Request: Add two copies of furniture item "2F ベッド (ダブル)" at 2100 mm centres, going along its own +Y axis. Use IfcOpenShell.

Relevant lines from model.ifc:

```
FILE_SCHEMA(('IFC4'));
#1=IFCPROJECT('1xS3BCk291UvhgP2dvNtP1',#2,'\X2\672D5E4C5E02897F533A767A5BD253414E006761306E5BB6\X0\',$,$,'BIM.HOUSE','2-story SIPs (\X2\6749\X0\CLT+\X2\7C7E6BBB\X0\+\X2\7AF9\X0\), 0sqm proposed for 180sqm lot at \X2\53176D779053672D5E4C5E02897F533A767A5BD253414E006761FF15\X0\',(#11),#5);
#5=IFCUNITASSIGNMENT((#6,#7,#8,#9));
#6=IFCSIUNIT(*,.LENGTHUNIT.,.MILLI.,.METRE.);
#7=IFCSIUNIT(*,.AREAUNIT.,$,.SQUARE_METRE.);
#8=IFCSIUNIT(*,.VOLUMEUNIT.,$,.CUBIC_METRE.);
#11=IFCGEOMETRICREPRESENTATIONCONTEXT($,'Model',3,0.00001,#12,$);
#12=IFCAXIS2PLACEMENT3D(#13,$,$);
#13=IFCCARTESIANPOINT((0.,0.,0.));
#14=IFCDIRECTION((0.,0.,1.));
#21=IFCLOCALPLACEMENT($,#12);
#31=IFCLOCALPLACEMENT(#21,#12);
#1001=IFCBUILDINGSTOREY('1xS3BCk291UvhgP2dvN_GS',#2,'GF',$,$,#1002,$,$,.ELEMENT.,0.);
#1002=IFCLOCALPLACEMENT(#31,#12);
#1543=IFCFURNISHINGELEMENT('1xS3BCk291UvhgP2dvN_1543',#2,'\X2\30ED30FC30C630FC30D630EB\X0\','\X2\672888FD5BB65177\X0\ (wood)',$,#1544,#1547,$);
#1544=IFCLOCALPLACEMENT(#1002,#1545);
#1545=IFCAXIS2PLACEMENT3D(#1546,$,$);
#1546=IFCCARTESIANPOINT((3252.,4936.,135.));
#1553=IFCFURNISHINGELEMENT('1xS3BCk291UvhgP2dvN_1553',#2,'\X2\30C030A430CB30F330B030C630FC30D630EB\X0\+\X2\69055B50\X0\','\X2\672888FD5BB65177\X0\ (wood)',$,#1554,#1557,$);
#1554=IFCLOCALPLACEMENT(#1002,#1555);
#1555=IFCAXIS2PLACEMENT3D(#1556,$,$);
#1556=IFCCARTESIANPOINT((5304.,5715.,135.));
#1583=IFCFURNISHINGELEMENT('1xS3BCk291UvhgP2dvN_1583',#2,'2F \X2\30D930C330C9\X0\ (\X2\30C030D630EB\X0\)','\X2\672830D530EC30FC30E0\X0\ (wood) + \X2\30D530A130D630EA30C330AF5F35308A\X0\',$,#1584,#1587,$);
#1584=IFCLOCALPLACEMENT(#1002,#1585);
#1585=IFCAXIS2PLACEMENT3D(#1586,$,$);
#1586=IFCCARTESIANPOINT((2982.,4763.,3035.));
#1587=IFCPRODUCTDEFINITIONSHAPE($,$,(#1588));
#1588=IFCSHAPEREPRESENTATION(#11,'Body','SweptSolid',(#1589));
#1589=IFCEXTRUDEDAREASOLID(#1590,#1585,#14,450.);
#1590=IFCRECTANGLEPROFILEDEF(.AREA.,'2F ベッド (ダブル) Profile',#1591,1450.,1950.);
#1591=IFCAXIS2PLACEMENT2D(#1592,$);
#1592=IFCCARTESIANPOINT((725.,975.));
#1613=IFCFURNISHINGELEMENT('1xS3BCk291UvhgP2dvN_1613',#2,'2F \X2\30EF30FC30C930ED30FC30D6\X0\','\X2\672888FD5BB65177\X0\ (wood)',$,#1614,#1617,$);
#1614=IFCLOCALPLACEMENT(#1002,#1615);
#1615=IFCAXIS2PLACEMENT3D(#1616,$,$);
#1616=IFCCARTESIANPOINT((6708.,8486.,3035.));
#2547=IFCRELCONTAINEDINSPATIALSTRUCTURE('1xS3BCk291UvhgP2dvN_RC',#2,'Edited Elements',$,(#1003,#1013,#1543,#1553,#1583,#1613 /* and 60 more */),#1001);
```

```python
import ifcopenshell
import ifcopenshell.api.geometry
import ifcopenshell.api.root
import ifcopenshell.util.element
import ifcopenshell.util.placement

model = ifcopenshell.open("model.ifc")


def reuse_history(source, copy):
    """copy_class also copies each property set's owner history, people and application; keep the originals."""
    for rel in copy.IsDefinedBy:
        if rel.is_a("IfcRelDefinesByProperties") and (history := rel.RelatingPropertyDefinition.OwnerHistory):
            rel.RelatingPropertyDefinition.OwnerHistory = source.OwnerHistory
            ifcopenshell.util.element.remove_deep2(model, history)


source = model.by_guid("1xS3BCk291UvhgP2dvN_1583")
base = ifcopenshell.util.placement.get_local_placement(source.ObjectPlacement)
step = base[:3, 1] * 2100.0

for i in range(1, 3):
    copy = ifcopenshell.api.root.copy_class(model, product=source)
    copy.Representation = ifcopenshell.util.element.copy_deep(
        model, source.Representation, exclude=["IfcGeometricRepresentationContext", "IfcRepresentationMap"]
    )
    reuse_history(source, copy)
    matrix = base.copy()
    matrix[:3, 3] += i * step
    print("added at", matrix[:3, 3].round(3) + 0.0)
    ifcopenshell.api.geometry.edit_object_placement(model, product=copy, matrix=matrix, is_si=False)

model.write("model_edited.ifc")
```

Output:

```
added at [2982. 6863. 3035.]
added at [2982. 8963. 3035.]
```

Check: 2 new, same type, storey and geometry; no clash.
